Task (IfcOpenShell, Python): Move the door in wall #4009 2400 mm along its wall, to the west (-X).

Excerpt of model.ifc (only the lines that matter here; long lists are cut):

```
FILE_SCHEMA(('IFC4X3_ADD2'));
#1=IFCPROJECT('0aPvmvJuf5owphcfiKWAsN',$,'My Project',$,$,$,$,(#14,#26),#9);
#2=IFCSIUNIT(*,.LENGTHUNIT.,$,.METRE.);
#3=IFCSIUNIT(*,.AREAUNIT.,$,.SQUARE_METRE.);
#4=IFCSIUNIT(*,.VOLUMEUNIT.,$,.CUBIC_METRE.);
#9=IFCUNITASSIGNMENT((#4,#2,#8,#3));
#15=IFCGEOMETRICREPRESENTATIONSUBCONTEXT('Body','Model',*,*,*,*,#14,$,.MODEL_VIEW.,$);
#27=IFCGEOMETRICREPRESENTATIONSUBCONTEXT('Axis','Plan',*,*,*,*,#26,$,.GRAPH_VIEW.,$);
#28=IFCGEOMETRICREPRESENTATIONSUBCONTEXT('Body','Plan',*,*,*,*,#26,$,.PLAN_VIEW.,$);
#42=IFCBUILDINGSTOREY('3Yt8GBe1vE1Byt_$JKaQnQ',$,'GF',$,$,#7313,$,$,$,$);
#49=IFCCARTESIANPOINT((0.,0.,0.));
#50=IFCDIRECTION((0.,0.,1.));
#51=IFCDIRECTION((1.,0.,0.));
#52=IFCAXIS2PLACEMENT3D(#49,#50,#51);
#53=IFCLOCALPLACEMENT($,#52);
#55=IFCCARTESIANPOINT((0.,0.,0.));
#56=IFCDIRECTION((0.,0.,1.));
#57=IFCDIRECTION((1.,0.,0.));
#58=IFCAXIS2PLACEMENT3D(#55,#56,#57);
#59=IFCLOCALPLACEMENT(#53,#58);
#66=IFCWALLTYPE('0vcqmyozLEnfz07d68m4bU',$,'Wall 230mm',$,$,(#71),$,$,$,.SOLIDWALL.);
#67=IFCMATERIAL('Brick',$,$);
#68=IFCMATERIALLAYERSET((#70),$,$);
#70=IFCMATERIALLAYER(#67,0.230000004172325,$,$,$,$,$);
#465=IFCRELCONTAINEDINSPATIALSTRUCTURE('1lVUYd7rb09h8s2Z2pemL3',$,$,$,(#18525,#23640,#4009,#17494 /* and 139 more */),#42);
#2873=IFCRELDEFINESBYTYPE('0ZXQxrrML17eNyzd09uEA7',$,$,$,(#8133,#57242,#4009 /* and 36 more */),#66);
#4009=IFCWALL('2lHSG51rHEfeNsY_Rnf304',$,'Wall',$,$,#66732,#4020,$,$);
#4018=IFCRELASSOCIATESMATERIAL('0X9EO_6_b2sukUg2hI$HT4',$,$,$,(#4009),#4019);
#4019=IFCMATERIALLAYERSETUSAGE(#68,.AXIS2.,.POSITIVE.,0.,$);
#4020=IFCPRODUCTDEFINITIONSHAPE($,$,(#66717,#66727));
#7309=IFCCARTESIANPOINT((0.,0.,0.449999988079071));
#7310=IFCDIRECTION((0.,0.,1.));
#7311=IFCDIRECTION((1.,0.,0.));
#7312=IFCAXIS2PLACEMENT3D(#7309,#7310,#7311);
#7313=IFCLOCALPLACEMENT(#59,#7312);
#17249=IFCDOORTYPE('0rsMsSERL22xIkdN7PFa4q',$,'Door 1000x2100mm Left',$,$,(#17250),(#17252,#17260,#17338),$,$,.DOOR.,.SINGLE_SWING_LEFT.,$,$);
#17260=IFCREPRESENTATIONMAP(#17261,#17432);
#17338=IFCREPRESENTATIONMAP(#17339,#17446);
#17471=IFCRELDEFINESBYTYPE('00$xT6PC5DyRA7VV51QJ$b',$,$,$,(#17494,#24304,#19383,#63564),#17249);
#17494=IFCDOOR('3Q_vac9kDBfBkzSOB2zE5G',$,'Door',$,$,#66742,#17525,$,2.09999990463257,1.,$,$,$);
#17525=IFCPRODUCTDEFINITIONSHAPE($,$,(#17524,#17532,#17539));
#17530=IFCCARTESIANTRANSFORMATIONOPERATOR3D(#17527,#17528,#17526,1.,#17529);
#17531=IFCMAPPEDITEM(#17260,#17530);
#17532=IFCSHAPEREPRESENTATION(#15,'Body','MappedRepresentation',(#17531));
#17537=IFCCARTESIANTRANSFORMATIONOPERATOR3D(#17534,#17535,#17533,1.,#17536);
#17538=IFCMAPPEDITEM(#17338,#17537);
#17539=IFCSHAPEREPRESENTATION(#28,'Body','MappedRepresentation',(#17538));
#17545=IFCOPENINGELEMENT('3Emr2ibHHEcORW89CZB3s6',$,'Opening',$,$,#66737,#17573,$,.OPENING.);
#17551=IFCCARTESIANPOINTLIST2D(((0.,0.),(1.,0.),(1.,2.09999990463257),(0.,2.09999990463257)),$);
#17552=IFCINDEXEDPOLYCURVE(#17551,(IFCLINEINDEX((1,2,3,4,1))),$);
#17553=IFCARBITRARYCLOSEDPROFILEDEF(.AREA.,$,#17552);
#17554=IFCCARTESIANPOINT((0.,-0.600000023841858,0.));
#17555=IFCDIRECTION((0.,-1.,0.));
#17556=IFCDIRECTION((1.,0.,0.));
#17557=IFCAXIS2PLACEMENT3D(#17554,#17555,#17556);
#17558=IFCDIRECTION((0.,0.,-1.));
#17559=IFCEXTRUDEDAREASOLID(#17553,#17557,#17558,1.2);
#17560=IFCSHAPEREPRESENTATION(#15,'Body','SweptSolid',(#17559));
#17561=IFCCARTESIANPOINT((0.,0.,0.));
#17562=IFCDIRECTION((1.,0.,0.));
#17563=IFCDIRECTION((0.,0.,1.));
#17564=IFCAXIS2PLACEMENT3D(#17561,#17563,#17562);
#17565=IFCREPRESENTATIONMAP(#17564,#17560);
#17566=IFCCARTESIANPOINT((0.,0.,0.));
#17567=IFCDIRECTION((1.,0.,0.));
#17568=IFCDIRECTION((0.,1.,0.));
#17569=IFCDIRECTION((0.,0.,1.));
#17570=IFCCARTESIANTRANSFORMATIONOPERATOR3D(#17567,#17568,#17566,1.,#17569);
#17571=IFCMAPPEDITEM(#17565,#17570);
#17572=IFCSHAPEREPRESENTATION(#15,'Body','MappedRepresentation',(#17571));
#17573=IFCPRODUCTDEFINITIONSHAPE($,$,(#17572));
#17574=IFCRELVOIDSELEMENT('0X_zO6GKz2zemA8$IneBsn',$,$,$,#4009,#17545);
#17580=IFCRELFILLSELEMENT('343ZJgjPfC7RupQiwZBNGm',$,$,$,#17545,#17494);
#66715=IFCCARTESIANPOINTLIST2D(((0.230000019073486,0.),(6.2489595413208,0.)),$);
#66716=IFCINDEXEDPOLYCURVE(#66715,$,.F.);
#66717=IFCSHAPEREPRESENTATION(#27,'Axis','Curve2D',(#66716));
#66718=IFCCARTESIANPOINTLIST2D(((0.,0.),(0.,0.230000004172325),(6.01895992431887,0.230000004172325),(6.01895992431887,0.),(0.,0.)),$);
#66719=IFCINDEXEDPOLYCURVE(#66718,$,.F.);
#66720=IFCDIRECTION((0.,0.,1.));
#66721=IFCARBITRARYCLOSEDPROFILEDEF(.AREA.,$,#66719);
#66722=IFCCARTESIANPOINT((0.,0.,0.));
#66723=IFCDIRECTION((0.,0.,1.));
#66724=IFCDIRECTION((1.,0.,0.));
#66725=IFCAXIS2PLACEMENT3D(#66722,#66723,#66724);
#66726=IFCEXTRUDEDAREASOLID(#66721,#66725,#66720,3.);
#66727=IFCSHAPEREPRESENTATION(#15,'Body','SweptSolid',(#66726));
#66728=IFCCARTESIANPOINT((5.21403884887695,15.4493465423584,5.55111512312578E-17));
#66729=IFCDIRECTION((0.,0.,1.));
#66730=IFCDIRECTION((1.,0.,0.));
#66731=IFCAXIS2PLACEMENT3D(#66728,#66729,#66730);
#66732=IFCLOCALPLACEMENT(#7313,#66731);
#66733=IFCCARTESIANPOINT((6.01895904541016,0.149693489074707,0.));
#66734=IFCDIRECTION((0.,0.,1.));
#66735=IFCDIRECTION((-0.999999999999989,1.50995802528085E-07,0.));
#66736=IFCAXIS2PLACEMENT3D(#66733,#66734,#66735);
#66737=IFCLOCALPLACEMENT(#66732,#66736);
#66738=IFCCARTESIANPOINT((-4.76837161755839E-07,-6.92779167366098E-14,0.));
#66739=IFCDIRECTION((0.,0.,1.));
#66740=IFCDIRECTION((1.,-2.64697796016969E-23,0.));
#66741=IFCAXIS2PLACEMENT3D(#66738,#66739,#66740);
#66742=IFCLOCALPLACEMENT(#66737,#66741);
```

```python
import ifcopenshell
import ifcopenshell.api.geometry
import ifcopenshell.util.placement

model = ifcopenshell.open("model.ifc")

door = model.by_guid("3Q_vac9kDBfBkzSOB2zE5G")
opening = door.FillsVoids[0].RelatingOpeningElement
wall = opening.VoidsElements[0].RelatingBuildingElement

wall_matrix = ifcopenshell.util.placement.get_local_placement(wall.ObjectPlacement)
shift = wall_matrix[:3, 0] * -2.4
before = ifcopenshell.util.placement.get_local_placement(door.ObjectPlacement)[:3, 3].copy()

# The door is placed relative to its opening, so it follows when the opening moves.
matrix = ifcopenshell.util.placement.get_local_placement(opening.ObjectPlacement)
matrix[:3, 3] += shift
ifcopenshell.api.geometry.edit_object_placement(
    model, product=opening, matrix=matrix, is_si=False, should_transform_children=True
)

after = ifcopenshell.util.placement.get_local_placement(door.ObjectPlacement)[:3, 3]
print("door moved by", (after - before).round(3) + 0.0)

model.write("model-out.ifc")
```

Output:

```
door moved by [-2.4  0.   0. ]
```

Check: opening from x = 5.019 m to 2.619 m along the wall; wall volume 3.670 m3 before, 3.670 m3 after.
